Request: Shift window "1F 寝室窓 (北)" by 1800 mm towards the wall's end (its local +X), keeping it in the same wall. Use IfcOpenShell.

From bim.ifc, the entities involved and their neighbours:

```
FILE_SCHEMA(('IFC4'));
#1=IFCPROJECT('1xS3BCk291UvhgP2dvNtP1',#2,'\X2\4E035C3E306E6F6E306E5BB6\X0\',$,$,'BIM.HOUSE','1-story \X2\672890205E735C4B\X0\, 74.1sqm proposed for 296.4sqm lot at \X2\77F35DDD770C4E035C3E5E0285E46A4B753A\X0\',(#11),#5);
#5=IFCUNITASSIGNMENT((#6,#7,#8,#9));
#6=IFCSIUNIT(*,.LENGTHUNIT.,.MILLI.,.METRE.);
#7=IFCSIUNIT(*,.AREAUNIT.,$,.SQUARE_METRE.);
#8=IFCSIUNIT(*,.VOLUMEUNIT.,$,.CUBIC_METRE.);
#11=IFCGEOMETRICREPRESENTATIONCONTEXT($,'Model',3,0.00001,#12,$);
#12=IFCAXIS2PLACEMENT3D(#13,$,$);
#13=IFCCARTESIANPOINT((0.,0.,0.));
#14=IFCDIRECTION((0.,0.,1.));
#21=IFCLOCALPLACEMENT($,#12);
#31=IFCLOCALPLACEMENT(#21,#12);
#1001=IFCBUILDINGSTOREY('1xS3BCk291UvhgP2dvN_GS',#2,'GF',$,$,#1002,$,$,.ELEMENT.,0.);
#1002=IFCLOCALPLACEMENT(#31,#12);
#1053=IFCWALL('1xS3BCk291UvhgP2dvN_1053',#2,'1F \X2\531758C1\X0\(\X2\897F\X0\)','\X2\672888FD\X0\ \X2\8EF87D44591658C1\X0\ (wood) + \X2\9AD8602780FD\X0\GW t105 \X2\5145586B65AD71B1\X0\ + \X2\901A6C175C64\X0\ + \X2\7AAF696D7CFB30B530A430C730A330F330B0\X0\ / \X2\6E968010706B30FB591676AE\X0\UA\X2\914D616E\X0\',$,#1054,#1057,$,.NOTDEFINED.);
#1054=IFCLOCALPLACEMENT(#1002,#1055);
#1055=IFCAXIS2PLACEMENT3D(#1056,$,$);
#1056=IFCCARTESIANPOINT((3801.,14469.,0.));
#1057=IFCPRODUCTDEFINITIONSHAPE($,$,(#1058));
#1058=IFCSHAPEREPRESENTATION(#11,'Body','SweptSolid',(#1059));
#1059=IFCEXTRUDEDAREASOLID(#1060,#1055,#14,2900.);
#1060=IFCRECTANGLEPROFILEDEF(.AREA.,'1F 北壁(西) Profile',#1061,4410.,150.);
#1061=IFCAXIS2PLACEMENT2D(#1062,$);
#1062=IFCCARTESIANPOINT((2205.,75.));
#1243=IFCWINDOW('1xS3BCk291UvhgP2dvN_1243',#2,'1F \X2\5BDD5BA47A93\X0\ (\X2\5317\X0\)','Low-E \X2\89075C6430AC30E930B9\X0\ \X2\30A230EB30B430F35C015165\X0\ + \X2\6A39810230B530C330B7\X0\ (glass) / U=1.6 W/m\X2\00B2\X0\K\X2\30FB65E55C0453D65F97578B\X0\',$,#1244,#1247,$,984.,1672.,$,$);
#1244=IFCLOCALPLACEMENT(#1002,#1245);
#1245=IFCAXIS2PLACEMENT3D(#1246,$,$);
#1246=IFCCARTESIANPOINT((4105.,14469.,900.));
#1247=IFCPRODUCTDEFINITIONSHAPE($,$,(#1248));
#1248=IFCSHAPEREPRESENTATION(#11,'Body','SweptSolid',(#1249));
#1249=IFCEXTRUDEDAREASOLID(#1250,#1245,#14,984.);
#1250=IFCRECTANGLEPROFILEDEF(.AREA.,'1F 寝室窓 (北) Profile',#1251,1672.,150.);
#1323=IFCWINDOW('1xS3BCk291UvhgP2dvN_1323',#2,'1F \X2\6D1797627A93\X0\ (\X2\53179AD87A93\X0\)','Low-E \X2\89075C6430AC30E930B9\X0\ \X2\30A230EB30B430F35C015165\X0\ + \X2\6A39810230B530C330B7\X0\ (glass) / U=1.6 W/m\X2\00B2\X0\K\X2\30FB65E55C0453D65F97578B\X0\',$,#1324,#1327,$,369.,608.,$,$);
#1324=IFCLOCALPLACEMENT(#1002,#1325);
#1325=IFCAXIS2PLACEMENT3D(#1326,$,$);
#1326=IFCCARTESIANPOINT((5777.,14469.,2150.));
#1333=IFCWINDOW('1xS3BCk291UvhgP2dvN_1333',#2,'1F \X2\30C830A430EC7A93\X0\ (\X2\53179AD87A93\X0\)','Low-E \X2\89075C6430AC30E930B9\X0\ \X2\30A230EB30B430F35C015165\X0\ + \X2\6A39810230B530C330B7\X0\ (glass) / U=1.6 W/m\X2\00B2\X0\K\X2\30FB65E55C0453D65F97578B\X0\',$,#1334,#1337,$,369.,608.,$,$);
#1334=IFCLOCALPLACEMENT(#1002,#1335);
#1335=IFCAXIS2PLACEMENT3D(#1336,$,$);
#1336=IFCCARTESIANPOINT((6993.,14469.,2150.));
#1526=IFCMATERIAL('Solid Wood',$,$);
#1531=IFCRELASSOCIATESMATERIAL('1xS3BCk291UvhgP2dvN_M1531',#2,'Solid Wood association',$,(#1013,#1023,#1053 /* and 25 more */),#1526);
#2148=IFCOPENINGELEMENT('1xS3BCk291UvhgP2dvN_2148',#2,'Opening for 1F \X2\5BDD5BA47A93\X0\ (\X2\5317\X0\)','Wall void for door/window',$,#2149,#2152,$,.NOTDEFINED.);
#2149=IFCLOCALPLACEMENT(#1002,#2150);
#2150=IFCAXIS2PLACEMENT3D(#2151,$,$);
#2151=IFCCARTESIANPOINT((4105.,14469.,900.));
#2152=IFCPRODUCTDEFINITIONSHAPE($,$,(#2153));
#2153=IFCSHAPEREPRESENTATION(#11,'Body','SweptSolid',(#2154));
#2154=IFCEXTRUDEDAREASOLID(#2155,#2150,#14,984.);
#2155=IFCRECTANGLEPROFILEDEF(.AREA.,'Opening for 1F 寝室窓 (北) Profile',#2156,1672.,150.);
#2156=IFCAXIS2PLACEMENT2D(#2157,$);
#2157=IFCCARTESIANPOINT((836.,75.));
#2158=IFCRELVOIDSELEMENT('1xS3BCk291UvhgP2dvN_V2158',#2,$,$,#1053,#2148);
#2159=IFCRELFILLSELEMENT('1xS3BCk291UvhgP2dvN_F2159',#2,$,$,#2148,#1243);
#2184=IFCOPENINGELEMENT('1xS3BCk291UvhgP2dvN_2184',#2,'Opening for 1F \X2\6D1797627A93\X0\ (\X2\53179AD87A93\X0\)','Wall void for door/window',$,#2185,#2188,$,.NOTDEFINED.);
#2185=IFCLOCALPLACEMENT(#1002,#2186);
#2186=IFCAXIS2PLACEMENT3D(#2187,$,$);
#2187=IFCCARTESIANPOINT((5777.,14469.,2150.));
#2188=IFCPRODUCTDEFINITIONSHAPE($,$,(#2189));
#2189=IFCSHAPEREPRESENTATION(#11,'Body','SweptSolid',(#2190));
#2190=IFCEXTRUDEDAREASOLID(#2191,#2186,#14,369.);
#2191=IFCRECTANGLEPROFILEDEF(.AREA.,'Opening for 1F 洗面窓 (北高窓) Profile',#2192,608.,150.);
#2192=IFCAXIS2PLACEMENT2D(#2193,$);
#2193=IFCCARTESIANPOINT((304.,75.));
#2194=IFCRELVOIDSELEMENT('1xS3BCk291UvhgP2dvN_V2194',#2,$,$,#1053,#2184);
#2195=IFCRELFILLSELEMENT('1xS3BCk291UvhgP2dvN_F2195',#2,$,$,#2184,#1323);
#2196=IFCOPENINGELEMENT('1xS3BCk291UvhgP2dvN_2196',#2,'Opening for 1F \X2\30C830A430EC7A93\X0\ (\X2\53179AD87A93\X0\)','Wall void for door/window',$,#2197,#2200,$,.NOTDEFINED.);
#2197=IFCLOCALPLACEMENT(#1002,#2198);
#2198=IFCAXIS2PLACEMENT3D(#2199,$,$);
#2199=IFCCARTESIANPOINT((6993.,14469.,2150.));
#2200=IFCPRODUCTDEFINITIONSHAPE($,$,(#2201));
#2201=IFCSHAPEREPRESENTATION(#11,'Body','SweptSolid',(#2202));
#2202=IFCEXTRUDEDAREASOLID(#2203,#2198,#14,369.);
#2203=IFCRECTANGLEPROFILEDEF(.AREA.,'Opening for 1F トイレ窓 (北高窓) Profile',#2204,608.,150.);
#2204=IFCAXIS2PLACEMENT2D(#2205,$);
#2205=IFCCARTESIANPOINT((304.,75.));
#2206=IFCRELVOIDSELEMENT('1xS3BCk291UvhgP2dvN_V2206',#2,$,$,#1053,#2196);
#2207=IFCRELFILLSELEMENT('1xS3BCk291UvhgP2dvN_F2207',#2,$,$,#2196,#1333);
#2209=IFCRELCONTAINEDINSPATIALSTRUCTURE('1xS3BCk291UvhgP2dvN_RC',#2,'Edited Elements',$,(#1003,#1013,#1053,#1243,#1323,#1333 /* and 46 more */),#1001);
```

```python
import ifcopenshell
import ifcopenshell.api.geometry
import ifcopenshell.util.placement
import ifcopenshell.util.unit

model = ifcopenshell.open("bim.ifc")
unit_scale = ifcopenshell.util.unit.calculate_unit_scale(model)

window = model.by_guid("1xS3BCk291UvhgP2dvN_1243")
opening = window.FillsVoids[0].RelatingOpeningElement
wall = opening.VoidsElements[0].RelatingBuildingElement

wall_matrix = ifcopenshell.util.placement.get_local_placement(wall.ObjectPlacement)
shift = wall_matrix[:3, 0] * 1.8 / unit_scale
before = ifcopenshell.util.placement.get_local_placement(window.ObjectPlacement)[:3, 3].copy()

# The window is not placed relative to its opening, so move both.
for product in (opening, window):
    matrix = ifcopenshell.util.placement.get_local_placement(product.ObjectPlacement)
    matrix[:3, 3] += shift
    ifcopenshell.api.geometry.edit_object_placement(model, product=product, matrix=matrix, is_si=False)

after = ifcopenshell.util.placement.get_local_placement(window.ObjectPlacement)[:3, 3]
print("window moved by", (after - before).round(3) + 0.0)

model.write("bim_v2.ifc")
```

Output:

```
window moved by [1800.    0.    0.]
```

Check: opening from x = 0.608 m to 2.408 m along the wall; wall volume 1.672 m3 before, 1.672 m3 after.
